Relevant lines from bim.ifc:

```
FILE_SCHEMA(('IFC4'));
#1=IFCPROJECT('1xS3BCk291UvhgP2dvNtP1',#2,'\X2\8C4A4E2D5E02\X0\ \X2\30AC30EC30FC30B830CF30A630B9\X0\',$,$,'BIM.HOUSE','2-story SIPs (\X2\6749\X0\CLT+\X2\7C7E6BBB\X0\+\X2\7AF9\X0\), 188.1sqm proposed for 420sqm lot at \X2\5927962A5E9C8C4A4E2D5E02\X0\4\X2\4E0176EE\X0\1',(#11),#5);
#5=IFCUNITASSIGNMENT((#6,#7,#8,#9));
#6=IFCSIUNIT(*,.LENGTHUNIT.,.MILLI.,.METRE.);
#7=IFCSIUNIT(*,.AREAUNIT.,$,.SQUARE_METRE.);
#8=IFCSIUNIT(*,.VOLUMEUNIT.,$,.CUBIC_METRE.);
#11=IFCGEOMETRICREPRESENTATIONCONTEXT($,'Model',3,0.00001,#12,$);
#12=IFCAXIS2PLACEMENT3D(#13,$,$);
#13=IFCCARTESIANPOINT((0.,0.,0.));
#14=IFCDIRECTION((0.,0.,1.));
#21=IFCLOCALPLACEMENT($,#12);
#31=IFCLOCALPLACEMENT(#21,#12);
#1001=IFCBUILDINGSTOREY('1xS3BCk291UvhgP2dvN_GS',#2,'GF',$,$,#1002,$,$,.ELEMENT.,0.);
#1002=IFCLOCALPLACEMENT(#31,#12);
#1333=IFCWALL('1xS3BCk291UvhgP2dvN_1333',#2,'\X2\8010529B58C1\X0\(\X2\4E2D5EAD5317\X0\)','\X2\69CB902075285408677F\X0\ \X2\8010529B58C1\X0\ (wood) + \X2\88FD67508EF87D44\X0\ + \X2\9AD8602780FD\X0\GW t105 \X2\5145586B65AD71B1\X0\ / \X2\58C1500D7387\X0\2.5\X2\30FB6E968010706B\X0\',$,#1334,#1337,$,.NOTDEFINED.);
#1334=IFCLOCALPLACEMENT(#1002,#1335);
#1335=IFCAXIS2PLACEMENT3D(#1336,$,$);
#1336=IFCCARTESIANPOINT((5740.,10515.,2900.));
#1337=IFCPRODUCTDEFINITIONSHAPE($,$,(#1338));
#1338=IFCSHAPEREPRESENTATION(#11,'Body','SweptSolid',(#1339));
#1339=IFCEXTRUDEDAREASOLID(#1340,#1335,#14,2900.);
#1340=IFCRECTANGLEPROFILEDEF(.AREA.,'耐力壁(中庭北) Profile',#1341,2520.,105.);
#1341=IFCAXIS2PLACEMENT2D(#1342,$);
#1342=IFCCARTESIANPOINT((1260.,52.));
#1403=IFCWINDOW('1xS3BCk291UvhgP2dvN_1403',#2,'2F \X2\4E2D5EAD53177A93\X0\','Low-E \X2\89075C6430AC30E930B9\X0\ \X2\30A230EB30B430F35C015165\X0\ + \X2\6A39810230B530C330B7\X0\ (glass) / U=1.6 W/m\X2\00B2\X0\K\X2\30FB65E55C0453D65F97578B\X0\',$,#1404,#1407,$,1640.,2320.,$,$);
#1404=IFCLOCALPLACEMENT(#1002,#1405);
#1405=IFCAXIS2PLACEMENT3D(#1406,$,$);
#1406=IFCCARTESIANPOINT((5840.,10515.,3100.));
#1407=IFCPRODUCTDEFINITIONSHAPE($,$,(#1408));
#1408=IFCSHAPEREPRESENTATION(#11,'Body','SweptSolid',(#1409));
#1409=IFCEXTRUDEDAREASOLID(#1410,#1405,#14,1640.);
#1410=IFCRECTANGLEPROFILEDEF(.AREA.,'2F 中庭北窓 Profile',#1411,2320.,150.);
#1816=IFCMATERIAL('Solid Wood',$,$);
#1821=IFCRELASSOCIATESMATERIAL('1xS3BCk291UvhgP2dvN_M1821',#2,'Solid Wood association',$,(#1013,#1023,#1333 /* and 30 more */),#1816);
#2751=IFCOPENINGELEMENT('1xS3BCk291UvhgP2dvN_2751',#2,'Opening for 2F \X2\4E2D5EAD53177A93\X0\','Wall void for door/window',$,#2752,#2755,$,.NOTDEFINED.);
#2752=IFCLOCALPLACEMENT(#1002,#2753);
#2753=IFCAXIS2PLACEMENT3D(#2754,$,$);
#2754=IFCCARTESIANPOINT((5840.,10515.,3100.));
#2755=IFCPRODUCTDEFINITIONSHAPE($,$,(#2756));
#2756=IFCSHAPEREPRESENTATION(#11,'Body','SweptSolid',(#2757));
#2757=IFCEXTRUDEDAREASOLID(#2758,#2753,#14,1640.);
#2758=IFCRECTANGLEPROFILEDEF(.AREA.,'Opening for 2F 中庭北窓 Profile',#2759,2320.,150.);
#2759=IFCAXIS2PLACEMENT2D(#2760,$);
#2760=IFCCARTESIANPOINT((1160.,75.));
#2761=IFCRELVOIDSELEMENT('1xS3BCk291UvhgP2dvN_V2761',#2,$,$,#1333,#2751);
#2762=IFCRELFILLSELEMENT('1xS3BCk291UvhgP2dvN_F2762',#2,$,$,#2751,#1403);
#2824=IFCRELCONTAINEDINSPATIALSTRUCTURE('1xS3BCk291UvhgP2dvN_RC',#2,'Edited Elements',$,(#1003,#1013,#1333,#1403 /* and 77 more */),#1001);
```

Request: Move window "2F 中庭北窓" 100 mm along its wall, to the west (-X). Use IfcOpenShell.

```python
import ifcopenshell
import ifcopenshell.api.geometry
import ifcopenshell.util.placement

model = ifcopenshell.open("bim.ifc")

window = model.by_guid("1xS3BCk291UvhgP2dvN_1403")
opening = window.FillsVoids[0].RelatingOpeningElement
wall = opening.VoidsElements[0].RelatingBuildingElement

wall_matrix = ifcopenshell.util.placement.get_local_placement(wall.ObjectPlacement)
shift = wall_matrix[:3, 0] * -100.0
before = ifcopenshell.util.placement.get_local_placement(window.ObjectPlacement)[:3, 3].copy()

# The window is not placed relative to its opening, so move both.
for product in (opening, window):
    matrix = ifcopenshell.util.placement.get_local_placement(product.ObjectPlacement)
    matrix[:3, 3] += shift
    ifcopenshell.api.geometry.edit_object_placement(model, product=product, matrix=matrix, is_si=False)

after = ifcopenshell.util.placement.get_local_placement(window.ObjectPlacement)[:3, 3]
print("window moved by", (after - before).round(3) + 0.0)

model.write("bim-out.ifc")
```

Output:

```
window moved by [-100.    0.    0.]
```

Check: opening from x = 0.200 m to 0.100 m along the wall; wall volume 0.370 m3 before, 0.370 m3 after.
